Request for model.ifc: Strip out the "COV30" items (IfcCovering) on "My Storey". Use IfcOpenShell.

First a look at what the model holds.

```python
import ifcopenshell
import ifcopenshell.util.element

model = ifcopenshell.open("model.ifc")
print(model.schema)
storey = next(s for s in model.by_type("IfcBuildingStorey") if s.Name == "My Storey")
coverings = [e for e in ifcopenshell.util.element.get_decomposition(storey) if e.is_a("IfcCovering")]
seen = {}
for e in coverings:
    element_type = ifcopenshell.util.element.get_type(e)
    name = element_type.Name if element_type not in (None, e) else None
    seen[name] = seen.get(name, 0) + 1
for name, count in sorted(seen.items(), key=str):
    print(count, "x", name)
```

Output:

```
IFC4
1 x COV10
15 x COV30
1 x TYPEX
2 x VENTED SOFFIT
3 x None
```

```python
import ifcopenshell
import ifcopenshell.api.root
import ifcopenshell.util.element

model = ifcopenshell.open("model.ifc")

storey = next(s for s in model.by_type("IfcBuildingStorey") if s.Name == "My Storey")
coverings = [e for e in ifcopenshell.util.element.get_decomposition(storey) if e.is_a("IfcCovering")]
targets = [e for e in coverings if (t := ifcopenshell.util.element.get_type(e)) not in (None, e) and t.Name == "COV30"]

for e in targets:
    ifcopenshell.api.root.remove_product(model, product=e)
print(len(targets), "removed")

model.write("model-out.ifc")
```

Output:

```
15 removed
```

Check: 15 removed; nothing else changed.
